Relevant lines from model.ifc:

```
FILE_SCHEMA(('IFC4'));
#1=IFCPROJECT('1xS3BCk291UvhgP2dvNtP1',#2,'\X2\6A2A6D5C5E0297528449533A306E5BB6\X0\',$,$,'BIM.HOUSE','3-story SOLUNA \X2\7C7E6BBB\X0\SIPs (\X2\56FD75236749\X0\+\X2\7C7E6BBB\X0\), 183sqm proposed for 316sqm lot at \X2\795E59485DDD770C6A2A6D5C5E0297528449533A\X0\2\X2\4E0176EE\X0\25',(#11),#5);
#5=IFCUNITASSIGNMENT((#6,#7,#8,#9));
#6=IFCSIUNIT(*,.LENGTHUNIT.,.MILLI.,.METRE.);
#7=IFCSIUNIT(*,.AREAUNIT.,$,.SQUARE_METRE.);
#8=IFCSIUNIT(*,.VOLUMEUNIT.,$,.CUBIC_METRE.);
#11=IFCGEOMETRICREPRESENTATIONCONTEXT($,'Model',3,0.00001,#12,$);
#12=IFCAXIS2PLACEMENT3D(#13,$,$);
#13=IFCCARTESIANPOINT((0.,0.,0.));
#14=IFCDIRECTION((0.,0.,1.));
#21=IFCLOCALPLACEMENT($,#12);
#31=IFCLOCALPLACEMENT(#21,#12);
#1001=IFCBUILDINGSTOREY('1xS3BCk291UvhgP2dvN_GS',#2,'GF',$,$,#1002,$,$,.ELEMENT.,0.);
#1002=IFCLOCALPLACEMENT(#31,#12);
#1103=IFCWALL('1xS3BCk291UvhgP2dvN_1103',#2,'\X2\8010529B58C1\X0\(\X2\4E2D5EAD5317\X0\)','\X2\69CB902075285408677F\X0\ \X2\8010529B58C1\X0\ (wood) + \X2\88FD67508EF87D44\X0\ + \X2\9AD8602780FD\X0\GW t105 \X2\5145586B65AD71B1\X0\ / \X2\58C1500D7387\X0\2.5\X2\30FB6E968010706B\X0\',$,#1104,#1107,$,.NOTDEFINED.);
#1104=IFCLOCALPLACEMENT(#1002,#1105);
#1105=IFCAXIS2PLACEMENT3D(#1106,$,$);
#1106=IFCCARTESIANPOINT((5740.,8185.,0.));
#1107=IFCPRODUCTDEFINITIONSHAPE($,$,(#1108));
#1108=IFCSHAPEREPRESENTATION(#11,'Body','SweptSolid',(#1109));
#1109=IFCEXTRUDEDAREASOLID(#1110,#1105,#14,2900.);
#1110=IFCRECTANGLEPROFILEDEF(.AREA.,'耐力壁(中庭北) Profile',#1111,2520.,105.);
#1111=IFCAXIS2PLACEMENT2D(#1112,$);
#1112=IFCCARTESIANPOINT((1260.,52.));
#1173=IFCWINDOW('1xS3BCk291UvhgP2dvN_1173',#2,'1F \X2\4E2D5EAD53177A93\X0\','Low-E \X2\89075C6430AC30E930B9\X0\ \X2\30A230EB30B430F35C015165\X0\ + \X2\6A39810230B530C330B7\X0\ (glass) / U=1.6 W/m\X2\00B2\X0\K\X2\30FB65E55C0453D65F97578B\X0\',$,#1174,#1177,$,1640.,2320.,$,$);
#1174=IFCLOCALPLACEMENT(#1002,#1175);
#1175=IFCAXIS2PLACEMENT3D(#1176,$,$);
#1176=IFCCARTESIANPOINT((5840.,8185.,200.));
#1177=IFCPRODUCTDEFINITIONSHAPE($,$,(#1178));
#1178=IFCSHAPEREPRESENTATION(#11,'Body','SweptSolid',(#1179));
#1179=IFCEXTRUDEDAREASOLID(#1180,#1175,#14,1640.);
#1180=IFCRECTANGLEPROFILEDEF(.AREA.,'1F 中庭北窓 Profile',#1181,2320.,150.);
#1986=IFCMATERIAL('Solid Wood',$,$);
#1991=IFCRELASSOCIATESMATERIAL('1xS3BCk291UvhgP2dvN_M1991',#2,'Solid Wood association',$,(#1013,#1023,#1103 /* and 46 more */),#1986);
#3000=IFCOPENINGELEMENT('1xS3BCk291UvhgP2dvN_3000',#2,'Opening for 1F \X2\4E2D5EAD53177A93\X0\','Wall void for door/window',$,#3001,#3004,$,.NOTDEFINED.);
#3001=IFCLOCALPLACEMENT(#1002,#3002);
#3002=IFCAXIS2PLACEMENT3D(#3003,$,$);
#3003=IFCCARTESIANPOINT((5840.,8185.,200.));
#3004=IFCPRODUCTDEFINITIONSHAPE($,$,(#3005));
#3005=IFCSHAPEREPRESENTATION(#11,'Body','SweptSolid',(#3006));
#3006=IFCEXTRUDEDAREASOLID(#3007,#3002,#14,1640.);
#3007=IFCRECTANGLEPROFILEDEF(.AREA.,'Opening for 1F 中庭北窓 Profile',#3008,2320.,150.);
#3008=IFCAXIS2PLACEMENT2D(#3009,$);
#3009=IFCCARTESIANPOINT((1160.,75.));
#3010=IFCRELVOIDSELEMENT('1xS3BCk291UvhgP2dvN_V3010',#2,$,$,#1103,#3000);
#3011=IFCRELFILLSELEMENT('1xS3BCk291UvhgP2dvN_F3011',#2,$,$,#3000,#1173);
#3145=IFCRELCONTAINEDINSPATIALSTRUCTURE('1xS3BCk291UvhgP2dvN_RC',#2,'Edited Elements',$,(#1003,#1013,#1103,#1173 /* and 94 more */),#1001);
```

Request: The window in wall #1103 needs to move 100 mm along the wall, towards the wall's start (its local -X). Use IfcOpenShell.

```python
import ifcopenshell
import ifcopenshell.api.geometry
import ifcopenshell.util.placement
import ifcopenshell.util.unit

model = ifcopenshell.open("model.ifc")
unit_scale = ifcopenshell.util.unit.calculate_unit_scale(model)

window = model.by_guid("1xS3BCk291UvhgP2dvN_1173")
opening = window.FillsVoids[0].RelatingOpeningElement
wall = opening.VoidsElements[0].RelatingBuildingElement

wall_matrix = ifcopenshell.util.placement.get_local_placement(wall.ObjectPlacement)
shift = wall_matrix[:3, 0] * -0.1 / unit_scale
before = ifcopenshell.util.placement.get_local_placement(window.ObjectPlacement)[:3, 3].copy()

# The window is not placed relative to its opening, so move both.
for product in (opening, window):
    matrix = ifcopenshell.util.placement.get_local_placement(product.ObjectPlacement)
    matrix[:3, 3] += shift
    ifcopenshell.api.geometry.edit_object_placement(model, product=product, matrix=matrix, is_si=False)

after = ifcopenshell.util.placement.get_local_placement(window.ObjectPlacement)[:3, 3]
print("window moved by", (after - before).round(3) + 0.0)

model.write("model_updated.ifc")
```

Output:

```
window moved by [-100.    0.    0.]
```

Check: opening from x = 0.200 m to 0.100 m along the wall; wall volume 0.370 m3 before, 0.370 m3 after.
